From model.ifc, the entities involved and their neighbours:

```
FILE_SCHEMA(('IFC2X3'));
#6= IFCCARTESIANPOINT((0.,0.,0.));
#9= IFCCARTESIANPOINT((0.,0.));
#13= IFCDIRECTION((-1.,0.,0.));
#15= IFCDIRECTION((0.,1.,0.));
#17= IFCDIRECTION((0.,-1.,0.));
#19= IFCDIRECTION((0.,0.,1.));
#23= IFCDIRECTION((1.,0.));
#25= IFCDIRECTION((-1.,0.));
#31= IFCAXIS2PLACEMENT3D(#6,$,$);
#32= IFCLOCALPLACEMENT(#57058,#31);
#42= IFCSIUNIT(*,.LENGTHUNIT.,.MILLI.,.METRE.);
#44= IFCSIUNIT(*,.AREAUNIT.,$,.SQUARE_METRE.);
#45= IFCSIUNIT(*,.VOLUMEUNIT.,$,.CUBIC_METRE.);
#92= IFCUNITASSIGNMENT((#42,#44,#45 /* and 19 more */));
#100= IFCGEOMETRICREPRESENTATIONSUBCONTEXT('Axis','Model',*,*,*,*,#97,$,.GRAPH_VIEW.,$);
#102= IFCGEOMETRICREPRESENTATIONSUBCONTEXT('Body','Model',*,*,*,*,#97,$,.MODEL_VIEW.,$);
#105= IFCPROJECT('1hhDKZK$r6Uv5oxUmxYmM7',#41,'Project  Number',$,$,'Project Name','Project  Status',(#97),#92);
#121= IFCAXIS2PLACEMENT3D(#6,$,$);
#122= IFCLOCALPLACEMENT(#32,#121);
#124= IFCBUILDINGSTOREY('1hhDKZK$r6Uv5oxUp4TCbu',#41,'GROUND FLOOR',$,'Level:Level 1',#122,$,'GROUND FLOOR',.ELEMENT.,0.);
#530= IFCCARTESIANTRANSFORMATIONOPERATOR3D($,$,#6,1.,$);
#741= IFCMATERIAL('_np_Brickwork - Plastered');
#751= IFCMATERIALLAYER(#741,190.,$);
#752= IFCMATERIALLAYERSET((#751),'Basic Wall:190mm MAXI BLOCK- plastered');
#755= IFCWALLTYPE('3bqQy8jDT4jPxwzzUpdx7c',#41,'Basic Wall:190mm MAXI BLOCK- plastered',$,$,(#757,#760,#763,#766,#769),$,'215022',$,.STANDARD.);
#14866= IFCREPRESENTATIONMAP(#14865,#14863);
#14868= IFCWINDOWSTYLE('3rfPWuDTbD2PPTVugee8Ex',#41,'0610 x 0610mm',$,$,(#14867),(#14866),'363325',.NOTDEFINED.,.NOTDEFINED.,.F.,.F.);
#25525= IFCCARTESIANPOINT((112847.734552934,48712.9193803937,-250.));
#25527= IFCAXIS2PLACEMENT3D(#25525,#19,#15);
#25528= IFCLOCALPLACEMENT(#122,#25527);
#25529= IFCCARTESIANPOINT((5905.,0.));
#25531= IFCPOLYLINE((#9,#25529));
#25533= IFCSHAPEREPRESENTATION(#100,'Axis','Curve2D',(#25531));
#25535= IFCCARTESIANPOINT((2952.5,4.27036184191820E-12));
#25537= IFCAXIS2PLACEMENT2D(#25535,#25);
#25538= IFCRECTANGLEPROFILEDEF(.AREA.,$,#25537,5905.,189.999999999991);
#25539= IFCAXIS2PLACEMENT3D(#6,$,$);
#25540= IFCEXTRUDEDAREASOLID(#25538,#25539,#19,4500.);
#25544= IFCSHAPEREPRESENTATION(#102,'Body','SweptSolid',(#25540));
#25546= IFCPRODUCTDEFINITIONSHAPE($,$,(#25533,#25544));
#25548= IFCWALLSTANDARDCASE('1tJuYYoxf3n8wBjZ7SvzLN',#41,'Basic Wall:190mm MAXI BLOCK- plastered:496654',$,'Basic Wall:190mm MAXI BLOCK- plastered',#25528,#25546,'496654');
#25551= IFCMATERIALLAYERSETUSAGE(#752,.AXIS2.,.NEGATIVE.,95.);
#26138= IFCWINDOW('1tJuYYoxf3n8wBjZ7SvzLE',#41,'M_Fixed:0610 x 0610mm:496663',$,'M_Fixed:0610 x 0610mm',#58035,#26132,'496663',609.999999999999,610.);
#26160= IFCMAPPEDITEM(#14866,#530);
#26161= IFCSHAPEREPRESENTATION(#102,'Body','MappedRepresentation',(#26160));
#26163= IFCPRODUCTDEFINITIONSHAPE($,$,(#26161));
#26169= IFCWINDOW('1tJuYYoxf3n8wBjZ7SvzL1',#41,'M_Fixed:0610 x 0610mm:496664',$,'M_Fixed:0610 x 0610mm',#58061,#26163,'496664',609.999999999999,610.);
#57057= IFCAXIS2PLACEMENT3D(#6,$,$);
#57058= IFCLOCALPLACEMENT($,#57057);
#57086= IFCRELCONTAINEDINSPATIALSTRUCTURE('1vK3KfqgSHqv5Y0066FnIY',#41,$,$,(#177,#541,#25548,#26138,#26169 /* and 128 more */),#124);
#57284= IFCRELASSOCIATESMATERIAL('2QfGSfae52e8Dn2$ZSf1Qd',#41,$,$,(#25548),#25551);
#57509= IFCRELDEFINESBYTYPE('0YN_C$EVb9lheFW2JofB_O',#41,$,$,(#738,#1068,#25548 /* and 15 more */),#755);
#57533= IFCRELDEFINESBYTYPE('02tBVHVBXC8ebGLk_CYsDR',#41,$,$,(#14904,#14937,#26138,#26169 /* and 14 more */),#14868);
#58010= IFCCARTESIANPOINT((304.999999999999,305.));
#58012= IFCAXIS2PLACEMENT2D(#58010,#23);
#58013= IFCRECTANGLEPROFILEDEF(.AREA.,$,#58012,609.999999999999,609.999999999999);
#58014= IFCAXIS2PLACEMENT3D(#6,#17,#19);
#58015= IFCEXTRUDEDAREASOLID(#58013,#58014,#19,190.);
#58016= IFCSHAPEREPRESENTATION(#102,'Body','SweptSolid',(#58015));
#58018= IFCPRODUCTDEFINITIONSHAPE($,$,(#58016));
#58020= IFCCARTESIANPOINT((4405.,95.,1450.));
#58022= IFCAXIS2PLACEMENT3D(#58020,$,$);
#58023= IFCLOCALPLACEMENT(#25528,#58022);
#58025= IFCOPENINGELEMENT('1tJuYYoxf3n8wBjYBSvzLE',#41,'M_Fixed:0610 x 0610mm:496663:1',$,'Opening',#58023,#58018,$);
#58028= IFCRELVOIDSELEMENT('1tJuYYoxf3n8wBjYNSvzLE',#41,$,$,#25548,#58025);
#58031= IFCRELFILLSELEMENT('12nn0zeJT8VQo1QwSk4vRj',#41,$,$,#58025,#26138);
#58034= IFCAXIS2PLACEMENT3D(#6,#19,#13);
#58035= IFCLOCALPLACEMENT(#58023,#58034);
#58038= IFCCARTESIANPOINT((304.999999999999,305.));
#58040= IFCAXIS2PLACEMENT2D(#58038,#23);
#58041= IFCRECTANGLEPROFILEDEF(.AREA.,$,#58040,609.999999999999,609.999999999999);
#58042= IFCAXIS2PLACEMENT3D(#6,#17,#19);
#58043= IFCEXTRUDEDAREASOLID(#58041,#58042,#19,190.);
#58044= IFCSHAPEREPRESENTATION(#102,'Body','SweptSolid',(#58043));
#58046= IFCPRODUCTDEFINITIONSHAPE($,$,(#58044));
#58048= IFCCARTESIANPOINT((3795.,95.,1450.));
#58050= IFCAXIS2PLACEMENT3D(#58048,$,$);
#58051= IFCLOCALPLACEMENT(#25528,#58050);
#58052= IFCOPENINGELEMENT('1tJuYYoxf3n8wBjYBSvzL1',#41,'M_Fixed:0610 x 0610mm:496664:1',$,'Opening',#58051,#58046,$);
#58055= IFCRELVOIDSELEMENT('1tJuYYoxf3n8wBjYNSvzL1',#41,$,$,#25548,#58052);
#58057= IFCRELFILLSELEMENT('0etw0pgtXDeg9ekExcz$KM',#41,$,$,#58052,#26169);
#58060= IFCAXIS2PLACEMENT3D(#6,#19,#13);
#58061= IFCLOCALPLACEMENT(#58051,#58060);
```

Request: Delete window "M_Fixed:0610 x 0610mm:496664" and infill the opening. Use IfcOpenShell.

```python
import ifcopenshell
import ifcopenshell.api.feature
import ifcopenshell.api.root
import ifcopenshell.geom
import ifcopenshell.util.shape

model = ifcopenshell.open("model.ifc")
settings = ifcopenshell.geom.settings()


def volume(element):
    """Net volume in cubic metres, openings subtracted."""
    shape = ifcopenshell.geom.create_shape(settings, element)
    return ifcopenshell.util.shape.get_volume(shape.geometry)


window = model.by_guid("1tJuYYoxf3n8wBjZ7SvzL1")
opening = window.FillsVoids[0].RelatingOpeningElement
wall = opening.VoidsElements[0].RelatingBuildingElement
before = volume(wall)

ifcopenshell.api.root.remove_product(model, product=window)
ifcopenshell.api.feature.remove_feature(model, feature=opening)

after = volume(wall)

print(f"wall volume {before:.3f} -> {after:.3f} m3")

model.write("model_updated.ifc")
```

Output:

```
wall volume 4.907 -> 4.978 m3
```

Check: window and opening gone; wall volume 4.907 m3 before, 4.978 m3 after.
